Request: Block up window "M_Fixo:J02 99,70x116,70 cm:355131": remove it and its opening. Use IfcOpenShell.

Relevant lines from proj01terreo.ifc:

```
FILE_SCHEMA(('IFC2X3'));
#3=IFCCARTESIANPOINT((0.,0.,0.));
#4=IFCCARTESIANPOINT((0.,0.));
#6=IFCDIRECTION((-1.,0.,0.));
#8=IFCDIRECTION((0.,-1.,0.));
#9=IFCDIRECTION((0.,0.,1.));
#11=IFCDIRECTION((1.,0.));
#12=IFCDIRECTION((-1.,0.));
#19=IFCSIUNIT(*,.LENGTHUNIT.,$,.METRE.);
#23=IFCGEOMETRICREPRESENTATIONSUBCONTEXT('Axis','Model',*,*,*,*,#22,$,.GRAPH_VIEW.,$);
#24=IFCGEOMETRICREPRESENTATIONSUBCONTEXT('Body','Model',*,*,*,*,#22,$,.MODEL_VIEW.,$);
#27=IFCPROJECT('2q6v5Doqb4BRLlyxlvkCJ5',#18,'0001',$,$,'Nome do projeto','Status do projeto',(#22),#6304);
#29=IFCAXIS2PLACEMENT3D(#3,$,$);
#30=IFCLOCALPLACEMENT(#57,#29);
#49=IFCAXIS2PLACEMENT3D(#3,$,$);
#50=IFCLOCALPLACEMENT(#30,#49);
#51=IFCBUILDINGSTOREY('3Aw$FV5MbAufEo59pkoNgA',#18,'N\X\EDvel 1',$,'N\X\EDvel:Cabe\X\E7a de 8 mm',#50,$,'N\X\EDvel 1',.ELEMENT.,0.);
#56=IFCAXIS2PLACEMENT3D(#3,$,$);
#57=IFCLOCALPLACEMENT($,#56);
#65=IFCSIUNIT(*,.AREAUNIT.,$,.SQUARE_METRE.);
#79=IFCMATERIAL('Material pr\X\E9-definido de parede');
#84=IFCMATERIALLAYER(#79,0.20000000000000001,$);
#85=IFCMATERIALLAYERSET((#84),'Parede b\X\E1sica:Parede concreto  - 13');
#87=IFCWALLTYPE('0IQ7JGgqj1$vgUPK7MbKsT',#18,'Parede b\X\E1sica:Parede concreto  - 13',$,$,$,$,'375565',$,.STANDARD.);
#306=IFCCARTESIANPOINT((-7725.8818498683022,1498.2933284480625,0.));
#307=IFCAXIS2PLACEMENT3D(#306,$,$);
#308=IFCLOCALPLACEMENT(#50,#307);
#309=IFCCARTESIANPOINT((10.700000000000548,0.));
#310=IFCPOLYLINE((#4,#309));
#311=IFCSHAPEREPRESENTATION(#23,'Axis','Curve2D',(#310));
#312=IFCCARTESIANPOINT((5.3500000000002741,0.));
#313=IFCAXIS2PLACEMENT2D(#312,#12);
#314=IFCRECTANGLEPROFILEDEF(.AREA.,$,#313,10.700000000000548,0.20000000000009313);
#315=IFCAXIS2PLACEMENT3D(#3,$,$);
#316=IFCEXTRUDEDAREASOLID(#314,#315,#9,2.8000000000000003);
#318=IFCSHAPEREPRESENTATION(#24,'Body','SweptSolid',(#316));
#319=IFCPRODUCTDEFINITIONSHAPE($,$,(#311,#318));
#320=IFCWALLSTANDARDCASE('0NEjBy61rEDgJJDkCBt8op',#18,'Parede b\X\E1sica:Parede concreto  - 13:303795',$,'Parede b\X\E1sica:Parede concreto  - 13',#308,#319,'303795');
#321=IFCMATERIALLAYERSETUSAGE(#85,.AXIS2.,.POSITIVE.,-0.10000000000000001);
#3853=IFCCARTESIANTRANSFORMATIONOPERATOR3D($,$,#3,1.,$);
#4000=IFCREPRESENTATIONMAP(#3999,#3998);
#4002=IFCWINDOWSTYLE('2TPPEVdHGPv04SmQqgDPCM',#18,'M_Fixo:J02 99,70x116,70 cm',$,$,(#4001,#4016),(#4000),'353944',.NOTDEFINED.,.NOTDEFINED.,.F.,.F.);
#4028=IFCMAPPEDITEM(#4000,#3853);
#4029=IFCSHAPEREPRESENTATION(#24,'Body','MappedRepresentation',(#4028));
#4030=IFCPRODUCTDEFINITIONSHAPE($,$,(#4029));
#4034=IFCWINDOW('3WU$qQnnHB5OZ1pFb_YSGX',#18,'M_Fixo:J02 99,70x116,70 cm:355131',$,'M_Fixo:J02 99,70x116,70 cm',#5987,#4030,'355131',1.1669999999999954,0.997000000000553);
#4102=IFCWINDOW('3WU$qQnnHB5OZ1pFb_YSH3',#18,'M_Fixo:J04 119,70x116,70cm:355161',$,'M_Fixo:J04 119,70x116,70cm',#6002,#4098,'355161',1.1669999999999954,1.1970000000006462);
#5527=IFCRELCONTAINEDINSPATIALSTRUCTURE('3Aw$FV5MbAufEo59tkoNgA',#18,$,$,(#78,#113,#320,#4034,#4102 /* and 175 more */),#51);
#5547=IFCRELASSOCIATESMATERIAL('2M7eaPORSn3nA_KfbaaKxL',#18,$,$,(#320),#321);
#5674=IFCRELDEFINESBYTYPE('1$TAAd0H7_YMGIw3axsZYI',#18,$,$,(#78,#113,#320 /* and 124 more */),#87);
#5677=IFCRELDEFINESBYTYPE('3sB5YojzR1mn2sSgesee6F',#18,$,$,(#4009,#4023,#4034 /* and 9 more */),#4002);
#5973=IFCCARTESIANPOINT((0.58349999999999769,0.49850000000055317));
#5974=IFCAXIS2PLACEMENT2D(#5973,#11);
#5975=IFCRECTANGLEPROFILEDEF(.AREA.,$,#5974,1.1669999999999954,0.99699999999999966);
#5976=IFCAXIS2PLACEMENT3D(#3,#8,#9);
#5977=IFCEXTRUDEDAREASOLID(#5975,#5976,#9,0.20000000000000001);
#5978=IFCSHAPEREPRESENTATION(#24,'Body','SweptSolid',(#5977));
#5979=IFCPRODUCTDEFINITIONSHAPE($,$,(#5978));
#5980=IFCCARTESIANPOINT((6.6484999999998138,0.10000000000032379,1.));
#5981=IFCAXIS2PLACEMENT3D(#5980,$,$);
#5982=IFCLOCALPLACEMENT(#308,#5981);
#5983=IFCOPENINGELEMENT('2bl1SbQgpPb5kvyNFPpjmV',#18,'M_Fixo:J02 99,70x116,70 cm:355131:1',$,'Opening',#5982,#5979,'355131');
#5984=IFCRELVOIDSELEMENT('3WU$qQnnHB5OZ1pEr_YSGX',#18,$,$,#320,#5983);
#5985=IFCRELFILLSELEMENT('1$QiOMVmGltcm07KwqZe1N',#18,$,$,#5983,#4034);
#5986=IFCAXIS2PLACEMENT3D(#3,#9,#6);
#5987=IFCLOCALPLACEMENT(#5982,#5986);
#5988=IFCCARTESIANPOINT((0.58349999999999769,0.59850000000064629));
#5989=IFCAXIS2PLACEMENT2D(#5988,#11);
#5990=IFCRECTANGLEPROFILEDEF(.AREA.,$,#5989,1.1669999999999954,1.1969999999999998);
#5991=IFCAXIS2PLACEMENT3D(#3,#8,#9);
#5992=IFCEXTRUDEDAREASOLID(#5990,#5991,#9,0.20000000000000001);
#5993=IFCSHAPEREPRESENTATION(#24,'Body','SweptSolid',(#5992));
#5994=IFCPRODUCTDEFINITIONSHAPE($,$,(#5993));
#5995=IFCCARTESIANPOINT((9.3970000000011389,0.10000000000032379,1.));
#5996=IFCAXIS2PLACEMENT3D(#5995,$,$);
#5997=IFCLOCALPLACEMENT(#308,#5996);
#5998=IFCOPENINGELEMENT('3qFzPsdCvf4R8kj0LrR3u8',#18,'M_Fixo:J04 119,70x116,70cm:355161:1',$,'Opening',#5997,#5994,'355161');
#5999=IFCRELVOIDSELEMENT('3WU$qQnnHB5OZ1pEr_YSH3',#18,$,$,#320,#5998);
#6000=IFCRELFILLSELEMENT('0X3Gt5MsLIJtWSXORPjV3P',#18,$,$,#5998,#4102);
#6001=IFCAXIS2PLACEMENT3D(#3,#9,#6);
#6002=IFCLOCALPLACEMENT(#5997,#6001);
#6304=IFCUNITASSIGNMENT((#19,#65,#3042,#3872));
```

```python
import ifcopenshell
import ifcopenshell.api.feature
import ifcopenshell.api.root
import ifcopenshell.geom
import ifcopenshell.util.shape

model = ifcopenshell.open("proj01terreo.ifc")
settings = ifcopenshell.geom.settings()


def volume(element):
    """Net volume in cubic metres, openings subtracted."""
    shape = ifcopenshell.geom.create_shape(settings, element)
    return ifcopenshell.util.shape.get_volume(shape.geometry)


window = model.by_guid("3WU$qQnnHB5OZ1pFb_YSGX")
opening = window.FillsVoids[0].RelatingOpeningElement
wall = opening.VoidsElements[0].RelatingBuildingElement
before = volume(wall)

ifcopenshell.api.root.remove_product(model, product=window)
ifcopenshell.api.feature.remove_feature(model, feature=opening)

after = volume(wall)

print(f"wall volume {before:.3f} -> {after:.3f} m3")

model.write("proj01terreo_updated.ifc")
```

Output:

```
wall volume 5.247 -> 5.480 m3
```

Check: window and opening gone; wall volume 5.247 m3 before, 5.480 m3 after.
